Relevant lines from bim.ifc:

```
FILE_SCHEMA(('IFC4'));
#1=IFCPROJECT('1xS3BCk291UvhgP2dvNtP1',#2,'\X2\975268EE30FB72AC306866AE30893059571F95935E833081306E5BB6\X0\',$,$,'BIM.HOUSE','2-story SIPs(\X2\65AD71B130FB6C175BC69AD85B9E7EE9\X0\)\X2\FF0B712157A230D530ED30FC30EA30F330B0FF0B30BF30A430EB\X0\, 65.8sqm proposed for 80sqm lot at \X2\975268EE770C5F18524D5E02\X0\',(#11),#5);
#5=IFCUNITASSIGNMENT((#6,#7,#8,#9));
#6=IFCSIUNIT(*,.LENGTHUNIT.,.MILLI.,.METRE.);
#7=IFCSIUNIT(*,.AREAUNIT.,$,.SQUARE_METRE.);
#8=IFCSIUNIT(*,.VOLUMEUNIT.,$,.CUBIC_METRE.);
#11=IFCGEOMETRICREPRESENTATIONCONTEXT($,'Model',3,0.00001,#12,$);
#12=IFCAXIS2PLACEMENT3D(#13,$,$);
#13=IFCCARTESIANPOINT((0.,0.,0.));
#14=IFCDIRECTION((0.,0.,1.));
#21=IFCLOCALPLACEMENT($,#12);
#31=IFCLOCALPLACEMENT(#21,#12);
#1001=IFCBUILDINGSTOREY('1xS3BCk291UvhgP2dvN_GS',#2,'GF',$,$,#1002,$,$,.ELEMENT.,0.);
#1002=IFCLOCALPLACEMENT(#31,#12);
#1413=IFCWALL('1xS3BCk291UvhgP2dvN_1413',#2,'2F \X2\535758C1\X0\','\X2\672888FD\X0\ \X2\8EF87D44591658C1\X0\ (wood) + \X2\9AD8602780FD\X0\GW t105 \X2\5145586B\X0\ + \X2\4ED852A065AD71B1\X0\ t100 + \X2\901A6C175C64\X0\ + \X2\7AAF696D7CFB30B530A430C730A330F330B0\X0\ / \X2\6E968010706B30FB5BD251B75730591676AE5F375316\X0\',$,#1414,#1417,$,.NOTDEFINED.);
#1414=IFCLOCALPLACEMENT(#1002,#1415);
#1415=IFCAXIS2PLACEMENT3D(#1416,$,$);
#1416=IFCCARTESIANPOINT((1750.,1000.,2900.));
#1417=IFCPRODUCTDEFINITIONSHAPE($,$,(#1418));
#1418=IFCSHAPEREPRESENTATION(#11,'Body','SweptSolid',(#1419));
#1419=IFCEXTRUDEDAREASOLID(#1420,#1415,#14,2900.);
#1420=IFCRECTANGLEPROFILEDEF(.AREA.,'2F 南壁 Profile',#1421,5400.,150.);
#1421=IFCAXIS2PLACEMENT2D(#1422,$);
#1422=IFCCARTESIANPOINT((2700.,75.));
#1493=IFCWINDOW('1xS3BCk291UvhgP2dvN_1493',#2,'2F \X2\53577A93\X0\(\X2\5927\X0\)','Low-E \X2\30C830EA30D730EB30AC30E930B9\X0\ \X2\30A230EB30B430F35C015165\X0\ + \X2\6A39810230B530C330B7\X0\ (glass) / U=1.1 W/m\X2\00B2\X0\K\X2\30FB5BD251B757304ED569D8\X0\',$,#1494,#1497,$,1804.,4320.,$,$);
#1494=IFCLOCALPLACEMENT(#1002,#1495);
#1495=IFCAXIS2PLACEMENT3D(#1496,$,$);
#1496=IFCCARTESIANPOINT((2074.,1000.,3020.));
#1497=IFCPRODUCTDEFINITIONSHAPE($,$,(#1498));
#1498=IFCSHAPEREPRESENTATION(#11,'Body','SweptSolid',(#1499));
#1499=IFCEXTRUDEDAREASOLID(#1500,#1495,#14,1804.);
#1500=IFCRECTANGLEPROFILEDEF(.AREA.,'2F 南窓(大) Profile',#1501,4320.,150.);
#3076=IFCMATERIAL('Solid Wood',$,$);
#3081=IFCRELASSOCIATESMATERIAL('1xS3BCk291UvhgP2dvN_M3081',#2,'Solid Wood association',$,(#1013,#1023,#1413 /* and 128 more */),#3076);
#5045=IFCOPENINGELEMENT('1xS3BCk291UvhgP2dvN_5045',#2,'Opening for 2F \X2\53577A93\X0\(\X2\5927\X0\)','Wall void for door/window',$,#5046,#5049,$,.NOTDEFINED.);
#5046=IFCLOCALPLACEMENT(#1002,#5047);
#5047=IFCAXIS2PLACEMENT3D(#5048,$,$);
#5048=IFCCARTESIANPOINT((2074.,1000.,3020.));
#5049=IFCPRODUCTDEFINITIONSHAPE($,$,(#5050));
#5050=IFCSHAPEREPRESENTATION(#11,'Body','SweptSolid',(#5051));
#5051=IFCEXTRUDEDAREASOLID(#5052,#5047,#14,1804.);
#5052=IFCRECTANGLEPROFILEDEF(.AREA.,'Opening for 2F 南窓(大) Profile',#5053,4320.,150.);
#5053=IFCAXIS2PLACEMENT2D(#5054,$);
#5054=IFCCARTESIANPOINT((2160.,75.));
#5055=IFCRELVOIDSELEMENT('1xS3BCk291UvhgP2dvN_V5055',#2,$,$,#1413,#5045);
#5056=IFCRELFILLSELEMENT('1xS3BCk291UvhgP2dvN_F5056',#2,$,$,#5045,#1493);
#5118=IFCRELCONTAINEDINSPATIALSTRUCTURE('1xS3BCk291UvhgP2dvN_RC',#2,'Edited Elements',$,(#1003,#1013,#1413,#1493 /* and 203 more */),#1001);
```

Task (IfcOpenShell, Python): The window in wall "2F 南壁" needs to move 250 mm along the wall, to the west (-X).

```python
import ifcopenshell
import ifcopenshell.api.geometry
import ifcopenshell.util.placement
import ifcopenshell.util.unit

model = ifcopenshell.open("bim.ifc")
unit_scale = ifcopenshell.util.unit.calculate_unit_scale(model)

window = model.by_guid("1xS3BCk291UvhgP2dvN_1493")
opening = window.FillsVoids[0].RelatingOpeningElement
wall = opening.VoidsElements[0].RelatingBuildingElement

wall_matrix = ifcopenshell.util.placement.get_local_placement(wall.ObjectPlacement)
shift = wall_matrix[:3, 0] * -0.25 / unit_scale
before = ifcopenshell.util.placement.get_local_placement(window.ObjectPlacement)[:3, 3].copy()

# The window is not placed relative to its opening, so move both.
for product in (opening, window):
    matrix = ifcopenshell.util.placement.get_local_placement(product.ObjectPlacement)
    matrix[:3, 3] += shift
    ifcopenshell.api.geometry.edit_object_placement(model, product=product, matrix=matrix, is_si=False)

after = ifcopenshell.util.placement.get_local_placement(window.ObjectPlacement)[:3, 3]
print("window moved by", (after - before).round(3) + 0.0)

model.write("bim_edited.ifc")
```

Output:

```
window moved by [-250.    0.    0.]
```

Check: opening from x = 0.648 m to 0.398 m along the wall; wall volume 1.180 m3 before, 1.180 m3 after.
